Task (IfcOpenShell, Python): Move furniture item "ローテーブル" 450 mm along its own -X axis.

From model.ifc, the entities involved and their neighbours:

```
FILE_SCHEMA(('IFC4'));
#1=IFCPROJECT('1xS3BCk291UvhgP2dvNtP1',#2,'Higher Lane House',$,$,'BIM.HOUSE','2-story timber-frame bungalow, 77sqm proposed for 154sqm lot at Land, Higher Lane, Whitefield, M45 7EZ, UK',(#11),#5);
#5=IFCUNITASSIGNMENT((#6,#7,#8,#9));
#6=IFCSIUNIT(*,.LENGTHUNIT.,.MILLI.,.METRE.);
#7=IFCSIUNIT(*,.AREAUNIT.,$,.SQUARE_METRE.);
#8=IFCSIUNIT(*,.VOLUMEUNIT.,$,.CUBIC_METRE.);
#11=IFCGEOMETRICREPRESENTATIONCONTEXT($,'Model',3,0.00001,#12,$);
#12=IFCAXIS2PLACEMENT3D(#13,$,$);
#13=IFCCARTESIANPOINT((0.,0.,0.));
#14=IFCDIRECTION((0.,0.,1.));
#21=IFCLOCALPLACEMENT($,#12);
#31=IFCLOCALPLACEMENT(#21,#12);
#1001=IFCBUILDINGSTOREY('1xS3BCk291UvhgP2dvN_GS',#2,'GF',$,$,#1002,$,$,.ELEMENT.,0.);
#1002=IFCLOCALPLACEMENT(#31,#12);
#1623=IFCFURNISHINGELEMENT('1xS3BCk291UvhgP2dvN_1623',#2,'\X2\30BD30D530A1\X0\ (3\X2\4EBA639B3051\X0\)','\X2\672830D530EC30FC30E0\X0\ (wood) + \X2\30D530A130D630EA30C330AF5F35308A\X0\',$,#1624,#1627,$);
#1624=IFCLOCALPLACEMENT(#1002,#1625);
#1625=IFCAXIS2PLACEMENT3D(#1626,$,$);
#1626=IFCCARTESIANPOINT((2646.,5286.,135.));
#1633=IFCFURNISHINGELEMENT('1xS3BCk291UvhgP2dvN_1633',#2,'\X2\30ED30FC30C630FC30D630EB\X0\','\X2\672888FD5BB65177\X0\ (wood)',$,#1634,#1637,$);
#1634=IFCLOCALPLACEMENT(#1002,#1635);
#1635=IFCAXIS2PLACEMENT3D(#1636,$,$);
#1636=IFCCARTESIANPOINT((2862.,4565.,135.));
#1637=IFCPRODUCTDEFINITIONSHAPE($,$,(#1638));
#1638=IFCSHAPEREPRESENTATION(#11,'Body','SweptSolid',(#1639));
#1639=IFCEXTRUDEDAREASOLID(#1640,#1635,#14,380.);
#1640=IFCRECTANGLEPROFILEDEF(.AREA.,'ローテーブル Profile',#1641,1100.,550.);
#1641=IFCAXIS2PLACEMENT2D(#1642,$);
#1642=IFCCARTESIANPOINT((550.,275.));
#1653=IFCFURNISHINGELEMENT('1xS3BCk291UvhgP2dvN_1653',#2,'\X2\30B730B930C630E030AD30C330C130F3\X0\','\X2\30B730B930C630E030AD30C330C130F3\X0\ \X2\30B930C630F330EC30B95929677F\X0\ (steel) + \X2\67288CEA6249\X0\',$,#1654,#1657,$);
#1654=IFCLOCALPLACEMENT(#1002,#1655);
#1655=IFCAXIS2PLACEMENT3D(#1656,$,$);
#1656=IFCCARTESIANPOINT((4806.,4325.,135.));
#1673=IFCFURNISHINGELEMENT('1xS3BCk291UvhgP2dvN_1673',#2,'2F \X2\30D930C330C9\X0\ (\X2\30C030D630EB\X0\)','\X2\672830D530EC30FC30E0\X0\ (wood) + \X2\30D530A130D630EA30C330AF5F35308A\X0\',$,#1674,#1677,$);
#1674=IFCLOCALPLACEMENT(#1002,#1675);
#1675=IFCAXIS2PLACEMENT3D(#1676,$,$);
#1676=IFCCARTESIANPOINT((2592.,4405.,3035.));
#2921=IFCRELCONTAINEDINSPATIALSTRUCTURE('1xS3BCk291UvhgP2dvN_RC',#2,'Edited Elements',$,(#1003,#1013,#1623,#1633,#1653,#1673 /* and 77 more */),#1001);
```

```python
import ifcopenshell
import ifcopenshell.api.geometry
import ifcopenshell.util.placement

model = ifcopenshell.open("model.ifc")

item = model.by_guid("1xS3BCk291UvhgP2dvN_1633")
matrix = ifcopenshell.util.placement.get_local_placement(item.ObjectPlacement)
matrix[:3, 3] -= matrix[:3, 0] * 450.0
ifcopenshell.api.geometry.edit_object_placement(model, product=item, matrix=matrix, is_si=False)

print(ifcopenshell.util.placement.get_local_placement(item.ObjectPlacement).round(3) + 0.0)

model.write("model_v2.ifc")
```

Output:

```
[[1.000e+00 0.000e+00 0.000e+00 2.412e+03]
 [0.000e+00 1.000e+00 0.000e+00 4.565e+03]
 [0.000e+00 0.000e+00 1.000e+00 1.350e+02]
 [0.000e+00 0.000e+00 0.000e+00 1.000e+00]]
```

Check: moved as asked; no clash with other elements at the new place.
